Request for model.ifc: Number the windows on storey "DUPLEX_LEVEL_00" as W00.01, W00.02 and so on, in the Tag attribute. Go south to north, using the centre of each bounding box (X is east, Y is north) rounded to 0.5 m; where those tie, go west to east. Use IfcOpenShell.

First a look at what the model holds.

```python
import ifcopenshell
import ifcopenshell.util.element
import ifcopenshell.util.placement

model = ifcopenshell.open("model.ifc")
print(model.schema)
storey = next(s for s in model.by_type("IfcBuildingStorey") if s.Name == "DUPLEX_LEVEL_00")
windows = [e for e in ifcopenshell.util.element.get_decomposition(storey) if e.is_a("IfcWindow")]
for e in sorted(windows, key=lambda e: e.id()):
    origin = ifcopenshell.util.placement.get_local_placement(e.ObjectPlacement)[:3, 3]
    print(e.id(), e.Tag, e.Name, origin.round(2) + 0.0, sep=" | ")
```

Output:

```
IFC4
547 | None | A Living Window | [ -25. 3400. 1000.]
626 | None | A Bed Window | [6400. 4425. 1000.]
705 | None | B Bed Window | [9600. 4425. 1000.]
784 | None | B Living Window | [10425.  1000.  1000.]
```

```python
import ifcopenshell
import ifcopenshell.geom
import ifcopenshell.util.element
import ifcopenshell.util.shape

model = ifcopenshell.open("model.ifc")
settings = ifcopenshell.geom.settings()
settings.set("use-world-coords", True)


def centre(element):
    shape = ifcopenshell.geom.create_shape(settings, element)
    return ifcopenshell.util.shape.get_bbox_centroid(shape.geometry)


storey = next(s for s in model.by_type("IfcBuildingStorey") if s.Name == "DUPLEX_LEVEL_00")
windows = [e for e in ifcopenshell.util.element.get_decomposition(storey) if e.is_a("IfcWindow")]

# Insertion points can sit at a corner or the storey origin, so sort by the geometry (in metres).
centres = {e: centre(e) for e in windows}
windows.sort(key=lambda e: (round(centres[e][1] / 0.5), centres[e][0]))

for i, e in enumerate(windows, start=1):
    number = f"W00.{i:02d}"
    e.Tag = number
    print(e.id(), number)

model.write("model_v2.ifc")
```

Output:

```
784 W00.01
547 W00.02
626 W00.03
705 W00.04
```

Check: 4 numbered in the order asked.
